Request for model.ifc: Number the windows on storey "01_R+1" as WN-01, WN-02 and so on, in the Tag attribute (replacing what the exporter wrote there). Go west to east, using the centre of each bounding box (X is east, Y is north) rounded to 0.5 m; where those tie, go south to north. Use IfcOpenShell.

First a look at what the model holds.

```python
import ifcopenshell
import ifcopenshell.util.element
import ifcopenshell.util.placement

model = ifcopenshell.open("model.ifc")
print(model.schema)
storey = next(s for s in model.by_type("IfcBuildingStorey") if s.Name == "01_R+1")
windows = [e for e in ifcopenshell.util.element.get_decomposition(storey) if e.is_a("IfcWindow")]
for e in sorted(windows, key=lambda e: e.id()):
    origin = ifcopenshell.util.placement.get_local_placement(e.ObjectPlacement)[:3, 3]
    print(e.id(), e.Tag, e.Name, origin.round(2) + 0.0, sep=" | ")
```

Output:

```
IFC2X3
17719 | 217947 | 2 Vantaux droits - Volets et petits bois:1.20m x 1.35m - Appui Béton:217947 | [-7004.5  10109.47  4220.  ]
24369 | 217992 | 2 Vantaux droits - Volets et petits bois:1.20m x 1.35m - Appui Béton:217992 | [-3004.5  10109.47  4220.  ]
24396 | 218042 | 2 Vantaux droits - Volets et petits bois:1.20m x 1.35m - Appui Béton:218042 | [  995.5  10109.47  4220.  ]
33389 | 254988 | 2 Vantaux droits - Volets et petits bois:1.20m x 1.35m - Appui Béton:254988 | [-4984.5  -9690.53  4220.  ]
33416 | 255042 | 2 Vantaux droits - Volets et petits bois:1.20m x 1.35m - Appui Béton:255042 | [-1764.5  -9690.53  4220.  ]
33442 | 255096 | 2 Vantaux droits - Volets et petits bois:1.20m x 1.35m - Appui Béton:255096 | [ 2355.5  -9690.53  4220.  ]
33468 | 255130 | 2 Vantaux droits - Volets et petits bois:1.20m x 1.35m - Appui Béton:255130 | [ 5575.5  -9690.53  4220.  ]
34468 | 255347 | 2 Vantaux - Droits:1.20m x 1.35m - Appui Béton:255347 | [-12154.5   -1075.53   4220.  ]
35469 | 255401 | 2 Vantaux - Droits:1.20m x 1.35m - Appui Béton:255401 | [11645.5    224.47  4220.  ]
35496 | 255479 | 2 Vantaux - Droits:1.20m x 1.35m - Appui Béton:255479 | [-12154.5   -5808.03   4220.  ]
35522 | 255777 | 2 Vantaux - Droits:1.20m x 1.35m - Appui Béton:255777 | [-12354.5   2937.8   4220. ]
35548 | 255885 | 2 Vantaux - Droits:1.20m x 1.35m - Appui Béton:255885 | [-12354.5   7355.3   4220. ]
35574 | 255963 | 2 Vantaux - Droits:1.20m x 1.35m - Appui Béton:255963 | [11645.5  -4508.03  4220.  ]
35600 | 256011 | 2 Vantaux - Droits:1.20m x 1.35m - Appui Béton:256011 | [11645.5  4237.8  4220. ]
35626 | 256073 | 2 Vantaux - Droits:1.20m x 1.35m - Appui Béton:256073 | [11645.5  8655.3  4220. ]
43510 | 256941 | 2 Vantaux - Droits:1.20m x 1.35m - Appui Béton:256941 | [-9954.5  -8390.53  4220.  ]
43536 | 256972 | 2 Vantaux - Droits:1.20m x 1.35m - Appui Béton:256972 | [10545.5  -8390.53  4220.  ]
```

```python
import ifcopenshell
import ifcopenshell.geom
import ifcopenshell.util.element
import ifcopenshell.util.shape

model = ifcopenshell.open("model.ifc")
settings = ifcopenshell.geom.settings()
settings.set("use-world-coords", True)


def centre(element):
    shape = ifcopenshell.geom.create_shape(settings, element)
    return ifcopenshell.util.shape.get_bbox_centroid(shape.geometry)


storey = next(s for s in model.by_type("IfcBuildingStorey") if s.Name == "01_R+1")
windows = [e for e in ifcopenshell.util.element.get_decomposition(storey) if e.is_a("IfcWindow")]

# Insertion points can sit at a corner or the storey origin, so sort by the geometry (in metres).
centres = {e: centre(e) for e in windows}
windows.sort(key=lambda e: (round(centres[e][0] / 0.5), centres[e][1]))

for i, e in enumerate(windows, start=1):
    number = f"WN-{i:02d}"
    e.Tag = number
    print(e.id(), number)

model.write("model_v2.ifc")
```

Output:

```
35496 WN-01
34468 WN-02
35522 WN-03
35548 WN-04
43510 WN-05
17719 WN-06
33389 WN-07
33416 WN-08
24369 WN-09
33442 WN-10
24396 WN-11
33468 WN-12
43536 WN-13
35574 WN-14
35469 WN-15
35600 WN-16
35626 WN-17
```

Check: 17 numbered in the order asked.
